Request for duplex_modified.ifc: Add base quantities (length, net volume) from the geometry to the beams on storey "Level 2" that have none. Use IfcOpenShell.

First a look at what the model holds.

```python
import ifcopenshell
import ifcopenshell.util.element
import ifcopenshell.util.unit

model = ifcopenshell.open("duplex_modified.ifc")
print(model.schema)
for unit_type in ("LENGTHUNIT", "AREAUNIT", "VOLUMEUNIT"):
    print(unit_type, ifcopenshell.util.unit.calculate_unit_scale(model, unit_type))
storey = next(s for s in model.by_type("IfcBuildingStorey") if s.Name == "Level 2")
beams = [e for e in ifcopenshell.util.element.get_decomposition(storey) if e.is_a("IfcBeam")]
for e in sorted(beams, key=lambda e: e.id()):
    print(e.id(), e.is_a(), e.Name, list(ifcopenshell.util.element.get_psets(e, qtos_only=True)), sep=" | ")
```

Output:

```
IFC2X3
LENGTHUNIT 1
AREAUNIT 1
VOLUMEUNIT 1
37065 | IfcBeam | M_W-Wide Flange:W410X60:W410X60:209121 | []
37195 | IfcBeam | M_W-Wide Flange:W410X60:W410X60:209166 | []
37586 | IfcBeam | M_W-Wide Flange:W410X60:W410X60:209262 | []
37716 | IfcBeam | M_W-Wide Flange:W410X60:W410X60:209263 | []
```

```python
import ifcopenshell
import ifcopenshell.api.pset
import ifcopenshell.geom
import ifcopenshell.util.element
import ifcopenshell.util.shape
import ifcopenshell.util.unit

model = ifcopenshell.open("duplex_modified.ifc")
unit_scale = ifcopenshell.util.unit.calculate_unit_scale(model)
volume_scale = ifcopenshell.util.unit.calculate_unit_scale(model, "VOLUMEUNIT")
settings = ifcopenshell.geom.settings()

storey = next(s for s in model.by_type("IfcBuildingStorey") if s.Name == "Level 2")
beams = [e for e in ifcopenshell.util.element.get_decomposition(storey) if e.is_a("IfcBeam")]

for e in sorted(beams, key=lambda e: e.id()):
    if ifcopenshell.util.element.get_psets(e, qtos_only=True, should_inherit=False):
        continue
    # Geometry comes back in metres, in the element's own axes.
    shape = ifcopenshell.geom.create_shape(settings, e)
    values = {
        "Length": ifcopenshell.util.shape.get_max_xyz(shape.geometry) / unit_scale,
        "NetVolume": ifcopenshell.util.shape.get_volume(shape.geometry) / volume_scale,
    }
    qto = ifcopenshell.api.pset.add_qto(model, product=e, name="BaseQuantities")
    ifcopenshell.api.pset.edit_qto(model, qto=qto, properties=values)
    print(e.id(), {k: round(v, 3) for k, v in values.items()})

model.write("duplex_modified_rev.ifc")
```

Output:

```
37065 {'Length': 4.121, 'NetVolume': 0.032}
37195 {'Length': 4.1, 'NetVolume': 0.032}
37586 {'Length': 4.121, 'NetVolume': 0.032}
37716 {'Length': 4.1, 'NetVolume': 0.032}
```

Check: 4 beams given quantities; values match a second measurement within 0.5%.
